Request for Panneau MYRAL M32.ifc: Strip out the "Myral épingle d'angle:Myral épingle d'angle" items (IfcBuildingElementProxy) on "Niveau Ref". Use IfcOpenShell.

First a look at what the model holds.

```python
import ifcopenshell
import ifcopenshell.util.element

model = ifcopenshell.open("Panneau MYRAL M32.ifc")
print(model.schema)
storey = next(s for s in model.by_type("IfcBuildingStorey") if s.Name == "Niveau Ref")
proxies = [e for e in ifcopenshell.util.element.get_decomposition(storey) if e.is_a("IfcBuildingElementProxy")]
seen = {}
for e in proxies:
    element_type = ifcopenshell.util.element.get_type(e)
    name = element_type.Name if element_type not in (None, e) else None
    seen[name] = seen.get(name, 0) + 1
for name, count in sorted(seen.items(), key=str):
    print(count, "x", name)
```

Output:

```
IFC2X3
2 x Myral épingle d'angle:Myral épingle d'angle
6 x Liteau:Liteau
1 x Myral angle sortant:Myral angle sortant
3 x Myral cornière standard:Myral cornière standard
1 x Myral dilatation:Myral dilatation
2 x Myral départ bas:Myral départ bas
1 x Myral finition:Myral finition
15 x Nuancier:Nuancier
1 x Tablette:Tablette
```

```python
import ifcopenshell
import ifcopenshell.api.root
import ifcopenshell.util.element

model = ifcopenshell.open("Panneau MYRAL M32.ifc")

storey = next(s for s in model.by_type("IfcBuildingStorey") if s.Name == "Niveau Ref")
proxies = [e for e in ifcopenshell.util.element.get_decomposition(storey) if e.is_a("IfcBuildingElementProxy")]
targets = [e for e in proxies if (t := ifcopenshell.util.element.get_type(e)) not in (None, e) and t.Name == "Myral épingle d'angle:Myral épingle d'angle"]

for e in targets:
    ifcopenshell.api.root.remove_product(model, product=e)
print(len(targets), "removed")

model.write("Panneau MYRAL M32_edited.ifc")
```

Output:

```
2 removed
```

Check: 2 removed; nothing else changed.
